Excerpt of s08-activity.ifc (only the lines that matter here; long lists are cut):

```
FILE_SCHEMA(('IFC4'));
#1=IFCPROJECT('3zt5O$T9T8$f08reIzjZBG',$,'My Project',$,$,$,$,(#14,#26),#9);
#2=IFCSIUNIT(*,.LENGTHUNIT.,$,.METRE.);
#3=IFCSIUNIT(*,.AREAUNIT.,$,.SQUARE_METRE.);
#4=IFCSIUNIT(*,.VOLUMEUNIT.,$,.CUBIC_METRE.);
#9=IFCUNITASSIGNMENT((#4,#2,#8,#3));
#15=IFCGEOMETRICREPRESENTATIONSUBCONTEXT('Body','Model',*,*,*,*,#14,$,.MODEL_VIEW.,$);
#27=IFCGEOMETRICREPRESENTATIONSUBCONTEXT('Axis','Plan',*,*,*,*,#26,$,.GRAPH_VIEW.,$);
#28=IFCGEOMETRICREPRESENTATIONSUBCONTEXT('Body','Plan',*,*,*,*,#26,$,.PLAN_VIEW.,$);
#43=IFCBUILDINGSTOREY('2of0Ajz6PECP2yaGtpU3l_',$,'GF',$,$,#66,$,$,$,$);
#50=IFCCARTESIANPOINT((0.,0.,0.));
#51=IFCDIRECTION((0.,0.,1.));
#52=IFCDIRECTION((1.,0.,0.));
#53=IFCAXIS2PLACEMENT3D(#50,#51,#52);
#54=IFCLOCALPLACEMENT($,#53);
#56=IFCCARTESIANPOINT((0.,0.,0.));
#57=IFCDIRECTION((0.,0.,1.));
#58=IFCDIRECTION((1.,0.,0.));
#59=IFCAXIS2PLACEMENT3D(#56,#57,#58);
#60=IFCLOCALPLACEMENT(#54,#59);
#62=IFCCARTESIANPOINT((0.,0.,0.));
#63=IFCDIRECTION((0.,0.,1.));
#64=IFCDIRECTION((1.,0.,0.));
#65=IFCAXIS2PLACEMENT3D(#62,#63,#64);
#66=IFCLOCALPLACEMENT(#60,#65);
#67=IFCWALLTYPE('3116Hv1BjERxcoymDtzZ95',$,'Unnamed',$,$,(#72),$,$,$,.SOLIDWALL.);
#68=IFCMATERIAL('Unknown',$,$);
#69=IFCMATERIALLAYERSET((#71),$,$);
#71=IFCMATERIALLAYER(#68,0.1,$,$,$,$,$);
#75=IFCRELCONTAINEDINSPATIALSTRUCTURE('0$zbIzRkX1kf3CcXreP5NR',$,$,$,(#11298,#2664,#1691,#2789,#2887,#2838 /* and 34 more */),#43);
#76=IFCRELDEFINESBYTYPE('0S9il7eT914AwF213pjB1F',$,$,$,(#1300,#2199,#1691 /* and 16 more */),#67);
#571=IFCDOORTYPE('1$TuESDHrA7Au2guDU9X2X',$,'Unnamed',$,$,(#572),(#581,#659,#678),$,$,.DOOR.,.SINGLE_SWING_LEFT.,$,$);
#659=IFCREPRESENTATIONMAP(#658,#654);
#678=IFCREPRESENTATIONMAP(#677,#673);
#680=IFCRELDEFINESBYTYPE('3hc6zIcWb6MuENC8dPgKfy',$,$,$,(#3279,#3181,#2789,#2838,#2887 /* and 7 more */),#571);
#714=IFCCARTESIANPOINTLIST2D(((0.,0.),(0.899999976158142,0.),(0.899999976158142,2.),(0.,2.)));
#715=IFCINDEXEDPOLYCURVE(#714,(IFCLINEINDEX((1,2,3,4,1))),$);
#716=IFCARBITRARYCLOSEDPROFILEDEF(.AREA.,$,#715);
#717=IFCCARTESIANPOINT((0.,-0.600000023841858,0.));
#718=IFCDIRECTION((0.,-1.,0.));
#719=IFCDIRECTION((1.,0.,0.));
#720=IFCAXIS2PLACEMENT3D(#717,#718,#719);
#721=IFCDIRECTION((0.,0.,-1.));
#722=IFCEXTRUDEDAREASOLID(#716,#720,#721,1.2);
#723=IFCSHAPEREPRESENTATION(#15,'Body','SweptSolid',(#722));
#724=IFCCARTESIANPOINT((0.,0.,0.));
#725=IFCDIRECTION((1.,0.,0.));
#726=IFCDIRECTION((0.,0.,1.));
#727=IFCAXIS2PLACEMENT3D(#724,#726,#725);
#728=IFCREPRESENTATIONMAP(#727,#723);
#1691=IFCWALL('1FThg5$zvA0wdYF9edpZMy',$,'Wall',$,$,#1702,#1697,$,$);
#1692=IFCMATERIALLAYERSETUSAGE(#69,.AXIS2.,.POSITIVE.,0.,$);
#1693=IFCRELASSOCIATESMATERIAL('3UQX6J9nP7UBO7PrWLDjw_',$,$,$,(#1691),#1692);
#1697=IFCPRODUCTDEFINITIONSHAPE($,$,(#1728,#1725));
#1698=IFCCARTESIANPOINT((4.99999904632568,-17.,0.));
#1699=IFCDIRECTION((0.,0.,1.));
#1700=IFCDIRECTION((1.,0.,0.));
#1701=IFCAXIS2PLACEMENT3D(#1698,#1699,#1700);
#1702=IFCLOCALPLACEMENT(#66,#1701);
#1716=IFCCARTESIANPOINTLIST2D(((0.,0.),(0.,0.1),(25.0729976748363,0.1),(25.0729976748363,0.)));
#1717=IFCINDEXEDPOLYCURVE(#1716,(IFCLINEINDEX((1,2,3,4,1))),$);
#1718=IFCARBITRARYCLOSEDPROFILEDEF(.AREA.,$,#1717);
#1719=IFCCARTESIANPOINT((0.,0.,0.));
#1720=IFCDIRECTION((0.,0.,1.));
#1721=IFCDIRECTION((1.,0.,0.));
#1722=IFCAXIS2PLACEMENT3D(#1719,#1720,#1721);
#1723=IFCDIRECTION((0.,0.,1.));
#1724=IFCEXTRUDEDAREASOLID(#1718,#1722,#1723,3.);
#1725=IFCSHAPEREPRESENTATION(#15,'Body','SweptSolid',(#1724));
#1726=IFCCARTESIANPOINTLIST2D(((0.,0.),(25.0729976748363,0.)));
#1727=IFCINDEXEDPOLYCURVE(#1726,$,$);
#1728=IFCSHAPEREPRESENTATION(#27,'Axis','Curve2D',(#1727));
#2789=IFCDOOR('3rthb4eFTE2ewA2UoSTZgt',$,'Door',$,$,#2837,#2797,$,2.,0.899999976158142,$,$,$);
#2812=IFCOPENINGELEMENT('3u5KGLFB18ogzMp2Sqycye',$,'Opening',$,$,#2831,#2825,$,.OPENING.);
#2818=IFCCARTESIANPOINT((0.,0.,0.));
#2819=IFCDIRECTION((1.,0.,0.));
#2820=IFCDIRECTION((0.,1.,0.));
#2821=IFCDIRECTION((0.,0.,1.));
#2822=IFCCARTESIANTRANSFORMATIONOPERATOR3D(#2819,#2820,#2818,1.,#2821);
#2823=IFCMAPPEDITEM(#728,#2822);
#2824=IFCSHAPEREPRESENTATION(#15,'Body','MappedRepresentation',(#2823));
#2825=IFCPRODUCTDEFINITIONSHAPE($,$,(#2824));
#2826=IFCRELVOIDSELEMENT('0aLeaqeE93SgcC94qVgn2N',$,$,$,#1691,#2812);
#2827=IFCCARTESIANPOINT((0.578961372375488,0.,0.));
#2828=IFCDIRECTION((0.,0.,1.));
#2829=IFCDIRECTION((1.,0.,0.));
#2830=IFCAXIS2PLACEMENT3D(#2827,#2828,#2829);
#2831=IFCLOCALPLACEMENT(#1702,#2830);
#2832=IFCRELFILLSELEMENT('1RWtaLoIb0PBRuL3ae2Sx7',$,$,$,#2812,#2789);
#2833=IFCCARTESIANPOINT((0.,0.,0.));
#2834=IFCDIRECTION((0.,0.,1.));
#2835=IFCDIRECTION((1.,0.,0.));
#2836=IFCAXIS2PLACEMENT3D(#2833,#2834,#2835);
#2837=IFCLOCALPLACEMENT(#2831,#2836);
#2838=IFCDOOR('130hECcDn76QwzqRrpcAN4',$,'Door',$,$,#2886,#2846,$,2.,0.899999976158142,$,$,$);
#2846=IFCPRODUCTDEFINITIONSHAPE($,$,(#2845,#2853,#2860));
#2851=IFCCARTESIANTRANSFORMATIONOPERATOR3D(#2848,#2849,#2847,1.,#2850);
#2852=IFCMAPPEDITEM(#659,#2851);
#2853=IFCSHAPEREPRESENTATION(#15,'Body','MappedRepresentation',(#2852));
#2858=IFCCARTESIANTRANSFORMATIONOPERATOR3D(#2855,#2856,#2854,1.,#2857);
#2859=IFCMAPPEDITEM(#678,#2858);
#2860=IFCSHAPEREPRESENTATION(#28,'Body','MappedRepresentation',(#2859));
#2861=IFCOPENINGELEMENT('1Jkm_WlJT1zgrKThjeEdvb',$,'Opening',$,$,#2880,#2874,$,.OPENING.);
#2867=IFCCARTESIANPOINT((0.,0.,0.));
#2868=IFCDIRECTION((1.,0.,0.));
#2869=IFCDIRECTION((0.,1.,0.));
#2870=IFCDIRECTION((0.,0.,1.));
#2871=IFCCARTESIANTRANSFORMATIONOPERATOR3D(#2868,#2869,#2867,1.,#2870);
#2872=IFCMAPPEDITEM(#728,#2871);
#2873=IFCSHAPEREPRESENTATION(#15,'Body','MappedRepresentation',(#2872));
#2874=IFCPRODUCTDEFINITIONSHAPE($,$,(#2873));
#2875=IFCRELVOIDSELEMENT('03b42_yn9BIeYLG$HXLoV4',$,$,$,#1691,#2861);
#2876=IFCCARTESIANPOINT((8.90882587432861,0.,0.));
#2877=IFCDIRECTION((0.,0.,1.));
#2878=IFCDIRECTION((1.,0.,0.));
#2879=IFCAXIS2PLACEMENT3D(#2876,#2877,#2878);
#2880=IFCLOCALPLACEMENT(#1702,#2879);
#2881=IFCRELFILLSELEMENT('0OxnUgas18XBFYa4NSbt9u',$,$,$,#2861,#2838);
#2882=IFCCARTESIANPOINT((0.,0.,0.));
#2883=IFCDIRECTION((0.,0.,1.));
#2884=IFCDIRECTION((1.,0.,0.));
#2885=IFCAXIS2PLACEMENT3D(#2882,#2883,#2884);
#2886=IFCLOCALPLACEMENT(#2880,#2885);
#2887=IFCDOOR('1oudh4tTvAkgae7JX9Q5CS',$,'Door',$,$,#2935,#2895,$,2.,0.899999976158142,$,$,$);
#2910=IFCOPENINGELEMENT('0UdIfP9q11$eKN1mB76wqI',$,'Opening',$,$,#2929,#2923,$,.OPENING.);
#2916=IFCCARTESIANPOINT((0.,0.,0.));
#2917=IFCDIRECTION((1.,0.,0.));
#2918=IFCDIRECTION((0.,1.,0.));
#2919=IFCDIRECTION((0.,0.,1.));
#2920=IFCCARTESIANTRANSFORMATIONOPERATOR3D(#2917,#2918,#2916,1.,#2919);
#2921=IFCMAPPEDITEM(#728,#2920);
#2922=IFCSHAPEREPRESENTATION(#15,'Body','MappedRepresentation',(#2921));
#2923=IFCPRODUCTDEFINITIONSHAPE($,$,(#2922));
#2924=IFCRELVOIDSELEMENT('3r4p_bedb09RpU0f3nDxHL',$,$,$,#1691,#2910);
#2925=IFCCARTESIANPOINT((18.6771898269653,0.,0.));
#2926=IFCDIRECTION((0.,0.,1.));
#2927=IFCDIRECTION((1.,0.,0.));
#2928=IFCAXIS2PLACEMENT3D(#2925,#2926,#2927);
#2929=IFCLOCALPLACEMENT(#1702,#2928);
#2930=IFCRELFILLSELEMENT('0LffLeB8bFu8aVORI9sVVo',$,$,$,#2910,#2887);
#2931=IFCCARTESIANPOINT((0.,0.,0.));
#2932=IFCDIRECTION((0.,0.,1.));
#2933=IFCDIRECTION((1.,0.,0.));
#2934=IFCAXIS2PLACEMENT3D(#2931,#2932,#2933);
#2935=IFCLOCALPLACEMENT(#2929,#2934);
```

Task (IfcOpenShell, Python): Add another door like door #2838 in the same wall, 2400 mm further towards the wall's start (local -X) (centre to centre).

```python
import ifcopenshell
import ifcopenshell.api.feature
import ifcopenshell.api.geometry
import ifcopenshell.api.root
import ifcopenshell.geom
import ifcopenshell.util.element
import ifcopenshell.util.placement
import ifcopenshell.util.shape
import ifcopenshell.util.unit

model = ifcopenshell.open("s08-activity.ifc")
unit_scale = ifcopenshell.util.unit.calculate_unit_scale(model)
settings = ifcopenshell.geom.settings()


def volume(element):
    """Net volume in cubic metres, openings subtracted."""
    shape = ifcopenshell.geom.create_shape(settings, element)
    return ifcopenshell.util.shape.get_volume(shape.geometry)


door = model.by_guid("130hECcDn76QwzqRrpcAN4")
opening = door.FillsVoids[0].RelatingOpeningElement
wall = opening.VoidsElements[0].RelatingBuildingElement
before = volume(wall)
shift = ifcopenshell.util.placement.get_local_placement(wall.ObjectPlacement)[:3, 0] * -2.4 / unit_scale

# copy_class copies the void relationship, type, container and properties, but no geometry.
new_opening = ifcopenshell.api.root.copy_class(model, product=opening)
new_opening.Representation = ifcopenshell.util.element.copy_deep(
    model, opening.Representation, exclude=["IfcGeometricRepresentationContext", "IfcRepresentationMap"]
)
new_door = ifcopenshell.api.root.copy_class(model, product=door)
new_door.Representation = ifcopenshell.util.element.copy_deep(
    model, door.Representation, exclude=["IfcGeometricRepresentationContext", "IfcRepresentationMap"]
)
ifcopenshell.api.feature.add_filling(model, opening=new_opening, element=new_door)

for old, new in ((opening, new_opening), (door, new_door)):
    matrix = ifcopenshell.util.placement.get_local_placement(old.ObjectPlacement)
    matrix[:3, 3] += shift
    ifcopenshell.api.geometry.edit_object_placement(model, product=new, matrix=matrix, is_si=False)

after = volume(wall)

print(f"wall volume {before:.3f} -> {after:.3f} m3")

model.write("s08-activity_edited.ifc")
```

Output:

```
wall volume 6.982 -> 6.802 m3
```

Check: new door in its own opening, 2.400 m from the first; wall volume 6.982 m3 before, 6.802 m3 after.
